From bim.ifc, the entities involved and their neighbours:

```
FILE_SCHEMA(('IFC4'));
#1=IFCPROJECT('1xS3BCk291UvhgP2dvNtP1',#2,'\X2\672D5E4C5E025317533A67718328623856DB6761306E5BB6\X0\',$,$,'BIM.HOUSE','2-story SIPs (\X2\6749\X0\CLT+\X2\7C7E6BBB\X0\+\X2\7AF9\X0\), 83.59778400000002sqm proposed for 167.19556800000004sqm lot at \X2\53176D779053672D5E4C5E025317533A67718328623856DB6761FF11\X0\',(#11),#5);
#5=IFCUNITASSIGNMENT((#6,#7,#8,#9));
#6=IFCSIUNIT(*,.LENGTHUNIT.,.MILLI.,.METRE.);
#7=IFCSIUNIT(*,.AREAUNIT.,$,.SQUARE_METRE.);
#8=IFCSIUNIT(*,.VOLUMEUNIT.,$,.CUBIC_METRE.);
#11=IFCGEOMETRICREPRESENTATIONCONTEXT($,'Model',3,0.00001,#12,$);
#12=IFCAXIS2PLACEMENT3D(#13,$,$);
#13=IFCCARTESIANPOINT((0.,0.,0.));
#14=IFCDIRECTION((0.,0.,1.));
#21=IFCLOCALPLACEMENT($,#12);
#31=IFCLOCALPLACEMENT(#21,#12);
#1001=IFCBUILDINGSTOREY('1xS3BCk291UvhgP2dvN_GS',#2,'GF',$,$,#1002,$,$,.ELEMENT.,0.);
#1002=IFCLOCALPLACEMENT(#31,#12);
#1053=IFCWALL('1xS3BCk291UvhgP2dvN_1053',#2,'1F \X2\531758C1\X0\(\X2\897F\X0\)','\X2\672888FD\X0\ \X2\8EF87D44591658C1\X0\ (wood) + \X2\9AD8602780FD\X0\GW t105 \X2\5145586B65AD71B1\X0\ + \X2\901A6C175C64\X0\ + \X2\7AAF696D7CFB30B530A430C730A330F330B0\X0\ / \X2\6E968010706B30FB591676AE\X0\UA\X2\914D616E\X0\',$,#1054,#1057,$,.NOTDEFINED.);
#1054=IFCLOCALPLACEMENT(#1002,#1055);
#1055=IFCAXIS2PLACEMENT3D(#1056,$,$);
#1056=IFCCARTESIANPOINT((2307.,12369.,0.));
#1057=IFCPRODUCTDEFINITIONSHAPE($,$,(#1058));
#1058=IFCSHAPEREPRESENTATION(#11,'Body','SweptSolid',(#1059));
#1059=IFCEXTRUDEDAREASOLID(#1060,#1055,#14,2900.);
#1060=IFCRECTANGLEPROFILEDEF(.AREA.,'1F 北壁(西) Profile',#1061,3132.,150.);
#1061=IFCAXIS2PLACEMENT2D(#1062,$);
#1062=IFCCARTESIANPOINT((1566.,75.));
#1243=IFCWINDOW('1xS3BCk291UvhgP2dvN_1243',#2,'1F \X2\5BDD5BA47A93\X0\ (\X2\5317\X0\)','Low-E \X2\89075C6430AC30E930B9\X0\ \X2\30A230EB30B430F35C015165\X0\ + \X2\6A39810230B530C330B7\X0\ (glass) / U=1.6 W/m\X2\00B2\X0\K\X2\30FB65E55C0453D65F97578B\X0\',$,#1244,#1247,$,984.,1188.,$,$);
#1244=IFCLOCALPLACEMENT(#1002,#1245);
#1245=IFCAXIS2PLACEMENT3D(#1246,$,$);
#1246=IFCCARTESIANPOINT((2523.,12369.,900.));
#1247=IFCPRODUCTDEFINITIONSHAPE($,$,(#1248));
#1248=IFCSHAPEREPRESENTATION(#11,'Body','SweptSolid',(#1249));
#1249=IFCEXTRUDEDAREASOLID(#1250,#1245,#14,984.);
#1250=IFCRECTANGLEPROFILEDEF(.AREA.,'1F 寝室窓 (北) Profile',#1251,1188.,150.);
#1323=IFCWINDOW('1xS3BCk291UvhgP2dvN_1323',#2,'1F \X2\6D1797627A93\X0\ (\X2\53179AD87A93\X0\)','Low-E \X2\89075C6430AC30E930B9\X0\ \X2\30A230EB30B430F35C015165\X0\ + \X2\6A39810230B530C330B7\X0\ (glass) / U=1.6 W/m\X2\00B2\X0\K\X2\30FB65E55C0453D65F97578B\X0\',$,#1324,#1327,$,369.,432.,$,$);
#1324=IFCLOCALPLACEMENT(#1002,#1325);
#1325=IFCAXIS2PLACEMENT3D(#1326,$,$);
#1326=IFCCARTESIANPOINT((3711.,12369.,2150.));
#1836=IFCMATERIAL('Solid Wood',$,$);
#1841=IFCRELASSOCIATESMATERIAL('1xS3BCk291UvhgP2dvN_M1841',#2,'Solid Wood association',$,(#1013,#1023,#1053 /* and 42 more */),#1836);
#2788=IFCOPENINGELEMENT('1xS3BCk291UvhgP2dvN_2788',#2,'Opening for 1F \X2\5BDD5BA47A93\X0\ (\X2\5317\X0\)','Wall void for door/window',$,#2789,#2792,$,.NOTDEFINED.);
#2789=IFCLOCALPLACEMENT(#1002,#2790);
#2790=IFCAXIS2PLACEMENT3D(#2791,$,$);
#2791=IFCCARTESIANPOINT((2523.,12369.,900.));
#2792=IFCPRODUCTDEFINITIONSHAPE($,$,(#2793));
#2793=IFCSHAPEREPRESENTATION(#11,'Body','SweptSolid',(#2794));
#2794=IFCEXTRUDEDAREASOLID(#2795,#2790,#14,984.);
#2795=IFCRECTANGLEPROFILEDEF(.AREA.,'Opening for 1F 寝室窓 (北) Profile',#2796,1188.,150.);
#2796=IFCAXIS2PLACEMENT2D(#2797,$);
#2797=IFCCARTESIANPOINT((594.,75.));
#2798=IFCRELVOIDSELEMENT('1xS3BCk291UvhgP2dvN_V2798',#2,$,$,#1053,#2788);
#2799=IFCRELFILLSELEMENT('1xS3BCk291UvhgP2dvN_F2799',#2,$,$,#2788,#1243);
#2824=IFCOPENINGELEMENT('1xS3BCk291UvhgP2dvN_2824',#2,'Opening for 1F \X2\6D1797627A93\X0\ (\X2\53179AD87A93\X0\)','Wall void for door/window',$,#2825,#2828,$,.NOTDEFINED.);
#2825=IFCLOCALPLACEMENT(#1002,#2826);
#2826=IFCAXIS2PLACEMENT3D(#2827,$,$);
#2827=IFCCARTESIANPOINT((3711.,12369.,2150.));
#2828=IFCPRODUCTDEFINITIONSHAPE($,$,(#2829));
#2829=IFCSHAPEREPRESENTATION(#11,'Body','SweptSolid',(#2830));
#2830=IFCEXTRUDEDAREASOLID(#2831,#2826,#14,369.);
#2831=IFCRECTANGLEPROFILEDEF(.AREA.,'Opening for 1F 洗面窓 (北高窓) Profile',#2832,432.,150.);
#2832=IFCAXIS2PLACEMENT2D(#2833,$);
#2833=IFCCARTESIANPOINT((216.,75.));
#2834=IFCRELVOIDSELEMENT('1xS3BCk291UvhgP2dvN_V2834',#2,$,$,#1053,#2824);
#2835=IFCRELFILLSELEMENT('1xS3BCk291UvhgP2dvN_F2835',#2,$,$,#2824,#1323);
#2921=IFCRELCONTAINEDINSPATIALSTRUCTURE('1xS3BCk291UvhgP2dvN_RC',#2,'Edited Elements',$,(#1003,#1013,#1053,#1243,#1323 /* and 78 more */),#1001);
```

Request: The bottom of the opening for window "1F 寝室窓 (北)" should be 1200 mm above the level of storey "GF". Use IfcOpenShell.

```python
import numpy as np
import ifcopenshell
import ifcopenshell.api.geometry
import ifcopenshell.geom
import ifcopenshell.util.element
import ifcopenshell.util.placement
import ifcopenshell.util.shape
import ifcopenshell.util.unit

model = ifcopenshell.open("bim.ifc")
unit_scale = ifcopenshell.util.unit.calculate_unit_scale(model)

window = model.by_id(1243)
opening = window.FillsVoids[0].RelatingOpeningElement
storey = ifcopenshell.util.element.get_container(window, ifc_class="IfcBuildingStorey")
level = ifcopenshell.util.placement.get_local_placement(storey.ObjectPlacement)[2, 3]

# The opening's origin need not be at the sill, so measure its lowest point.
shape = ifcopenshell.geom.create_shape(ifcopenshell.geom.settings(), opening)
bottom = ifcopenshell.util.shape.get_shape_bottom_elevation(shape, shape.geometry) / unit_scale
dz = level + 1.2 / unit_scale - bottom

shift = np.array([0.0, 0.0, dz])
# The window is not placed relative to its opening, so move both.
for product in (opening, window):
    matrix = ifcopenshell.util.placement.get_local_placement(product.ObjectPlacement)
    matrix[:3, 3] += shift
    ifcopenshell.api.geometry.edit_object_placement(model, product=product, matrix=matrix, is_si=False)

print(f"moved by {dz * unit_scale:+.3f} m")

model.write("bim_edited.ifc")
```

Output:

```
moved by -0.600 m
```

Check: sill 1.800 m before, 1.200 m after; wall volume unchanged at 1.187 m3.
